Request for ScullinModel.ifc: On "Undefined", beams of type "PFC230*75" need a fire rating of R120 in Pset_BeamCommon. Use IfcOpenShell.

First a look at what the model holds.

```python
import ifcopenshell
import ifcopenshell.util.element

model = ifcopenshell.open("ScullinModel.ifc")
print(model.schema)
storey = next(s for s in model.by_type("IfcBuildingStorey") if s.Name == "Undefined")
beams = [e for e in ifcopenshell.util.element.get_decomposition(storey) if e.is_a("IfcBeam")]
seen = {}
for e in beams:
    element_type = ifcopenshell.util.element.get_type(e)
    key = (element_type.Name if element_type != e and element_type else None, ifcopenshell.util.element.get_pset(e, "Pset_BeamCommon", "FireRating"))
    seen[key] = seen.get(key, 0) + 1
for (name, value), count in sorted(seen.items(), key=str):
    print(count, "x", name, "|", value)
```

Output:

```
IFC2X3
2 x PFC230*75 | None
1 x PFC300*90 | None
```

```python
import ifcopenshell
import ifcopenshell.api.pset
import ifcopenshell.util.element

model = ifcopenshell.open("ScullinModel.ifc")

storey = next(s for s in model.by_type("IfcBuildingStorey") if s.Name == "Undefined")
beams = [e for e in ifcopenshell.util.element.get_decomposition(storey) if e.is_a("IfcBeam")]

count = 0
for e in beams:
    element_type = ifcopenshell.util.element.get_type(e)
    if element_type in (None, e) or element_type.Name != "PFC230*75":
        continue
    found = ifcopenshell.util.element.get_pset(e, "Pset_BeamCommon", should_inherit=False)
    if found:
        pset = model.by_id(found["id"])
        if len(ifcopenshell.util.element.get_elements_by_pset(pset)) > 1:
            pset = ifcopenshell.api.pset.unshare_pset(model, products=[e], pset=pset)[0]
    else:
        pset = ifcopenshell.api.pset.add_pset(model, product=e, name="Pset_BeamCommon")
    ifcopenshell.api.pset.edit_pset(model, pset=pset, properties={"FireRating": "R120"})
    count += 1

print(count, "beams updated")

model.write("ScullinModel_v2.ifc")
```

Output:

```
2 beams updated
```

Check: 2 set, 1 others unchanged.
